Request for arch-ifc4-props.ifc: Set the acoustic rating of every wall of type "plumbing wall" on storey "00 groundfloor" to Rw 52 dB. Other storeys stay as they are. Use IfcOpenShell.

First a look at what the model holds.

```python
import ifcopenshell
import ifcopenshell.util.element

model = ifcopenshell.open("arch-ifc4-props.ifc")
print(model.schema)
storey = next(s for s in model.by_type("IfcBuildingStorey") if s.Name == "00 groundfloor")
walls = [e for e in ifcopenshell.util.element.get_decomposition(storey) if e.is_a("IfcWall")]
seen = {}
for e in walls:
    element_type = ifcopenshell.util.element.get_type(e)
    key = (element_type.Name if element_type != e and element_type else None, ifcopenshell.util.element.get_pset(e, "Pset_WallCommon", "AcousticRating"))
    seen[key] = seen.get(key, 0) + 1
for (name, value), count in sorted(seen.items(), key=str):
    print(count, "x", name, "|", value)
```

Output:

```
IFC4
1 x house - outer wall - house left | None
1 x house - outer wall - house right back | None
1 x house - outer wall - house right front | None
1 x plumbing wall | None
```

```python
import ifcopenshell
import ifcopenshell.api.pset
import ifcopenshell.util.element

model = ifcopenshell.open("arch-ifc4-props.ifc")

storey = next(s for s in model.by_type("IfcBuildingStorey") if s.Name == "00 groundfloor")
walls = [e for e in ifcopenshell.util.element.get_decomposition(storey) if e.is_a("IfcWall")]

count = 0
for e in walls:
    element_type = ifcopenshell.util.element.get_type(e)
    if element_type in (None, e) or element_type.Name != "plumbing wall":
        continue
    # add_pset returns the element's existing set when there is one.
    pset = ifcopenshell.api.pset.add_pset(model, product=e, name="Pset_WallCommon")
    ifcopenshell.api.pset.edit_pset(model, pset=pset, properties={"AcousticRating": "Rw 52 dB"})
    count += 1

print(count, "walls updated")

model.write("arch-ifc4-props_v2.ifc")
```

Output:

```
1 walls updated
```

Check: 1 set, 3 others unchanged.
